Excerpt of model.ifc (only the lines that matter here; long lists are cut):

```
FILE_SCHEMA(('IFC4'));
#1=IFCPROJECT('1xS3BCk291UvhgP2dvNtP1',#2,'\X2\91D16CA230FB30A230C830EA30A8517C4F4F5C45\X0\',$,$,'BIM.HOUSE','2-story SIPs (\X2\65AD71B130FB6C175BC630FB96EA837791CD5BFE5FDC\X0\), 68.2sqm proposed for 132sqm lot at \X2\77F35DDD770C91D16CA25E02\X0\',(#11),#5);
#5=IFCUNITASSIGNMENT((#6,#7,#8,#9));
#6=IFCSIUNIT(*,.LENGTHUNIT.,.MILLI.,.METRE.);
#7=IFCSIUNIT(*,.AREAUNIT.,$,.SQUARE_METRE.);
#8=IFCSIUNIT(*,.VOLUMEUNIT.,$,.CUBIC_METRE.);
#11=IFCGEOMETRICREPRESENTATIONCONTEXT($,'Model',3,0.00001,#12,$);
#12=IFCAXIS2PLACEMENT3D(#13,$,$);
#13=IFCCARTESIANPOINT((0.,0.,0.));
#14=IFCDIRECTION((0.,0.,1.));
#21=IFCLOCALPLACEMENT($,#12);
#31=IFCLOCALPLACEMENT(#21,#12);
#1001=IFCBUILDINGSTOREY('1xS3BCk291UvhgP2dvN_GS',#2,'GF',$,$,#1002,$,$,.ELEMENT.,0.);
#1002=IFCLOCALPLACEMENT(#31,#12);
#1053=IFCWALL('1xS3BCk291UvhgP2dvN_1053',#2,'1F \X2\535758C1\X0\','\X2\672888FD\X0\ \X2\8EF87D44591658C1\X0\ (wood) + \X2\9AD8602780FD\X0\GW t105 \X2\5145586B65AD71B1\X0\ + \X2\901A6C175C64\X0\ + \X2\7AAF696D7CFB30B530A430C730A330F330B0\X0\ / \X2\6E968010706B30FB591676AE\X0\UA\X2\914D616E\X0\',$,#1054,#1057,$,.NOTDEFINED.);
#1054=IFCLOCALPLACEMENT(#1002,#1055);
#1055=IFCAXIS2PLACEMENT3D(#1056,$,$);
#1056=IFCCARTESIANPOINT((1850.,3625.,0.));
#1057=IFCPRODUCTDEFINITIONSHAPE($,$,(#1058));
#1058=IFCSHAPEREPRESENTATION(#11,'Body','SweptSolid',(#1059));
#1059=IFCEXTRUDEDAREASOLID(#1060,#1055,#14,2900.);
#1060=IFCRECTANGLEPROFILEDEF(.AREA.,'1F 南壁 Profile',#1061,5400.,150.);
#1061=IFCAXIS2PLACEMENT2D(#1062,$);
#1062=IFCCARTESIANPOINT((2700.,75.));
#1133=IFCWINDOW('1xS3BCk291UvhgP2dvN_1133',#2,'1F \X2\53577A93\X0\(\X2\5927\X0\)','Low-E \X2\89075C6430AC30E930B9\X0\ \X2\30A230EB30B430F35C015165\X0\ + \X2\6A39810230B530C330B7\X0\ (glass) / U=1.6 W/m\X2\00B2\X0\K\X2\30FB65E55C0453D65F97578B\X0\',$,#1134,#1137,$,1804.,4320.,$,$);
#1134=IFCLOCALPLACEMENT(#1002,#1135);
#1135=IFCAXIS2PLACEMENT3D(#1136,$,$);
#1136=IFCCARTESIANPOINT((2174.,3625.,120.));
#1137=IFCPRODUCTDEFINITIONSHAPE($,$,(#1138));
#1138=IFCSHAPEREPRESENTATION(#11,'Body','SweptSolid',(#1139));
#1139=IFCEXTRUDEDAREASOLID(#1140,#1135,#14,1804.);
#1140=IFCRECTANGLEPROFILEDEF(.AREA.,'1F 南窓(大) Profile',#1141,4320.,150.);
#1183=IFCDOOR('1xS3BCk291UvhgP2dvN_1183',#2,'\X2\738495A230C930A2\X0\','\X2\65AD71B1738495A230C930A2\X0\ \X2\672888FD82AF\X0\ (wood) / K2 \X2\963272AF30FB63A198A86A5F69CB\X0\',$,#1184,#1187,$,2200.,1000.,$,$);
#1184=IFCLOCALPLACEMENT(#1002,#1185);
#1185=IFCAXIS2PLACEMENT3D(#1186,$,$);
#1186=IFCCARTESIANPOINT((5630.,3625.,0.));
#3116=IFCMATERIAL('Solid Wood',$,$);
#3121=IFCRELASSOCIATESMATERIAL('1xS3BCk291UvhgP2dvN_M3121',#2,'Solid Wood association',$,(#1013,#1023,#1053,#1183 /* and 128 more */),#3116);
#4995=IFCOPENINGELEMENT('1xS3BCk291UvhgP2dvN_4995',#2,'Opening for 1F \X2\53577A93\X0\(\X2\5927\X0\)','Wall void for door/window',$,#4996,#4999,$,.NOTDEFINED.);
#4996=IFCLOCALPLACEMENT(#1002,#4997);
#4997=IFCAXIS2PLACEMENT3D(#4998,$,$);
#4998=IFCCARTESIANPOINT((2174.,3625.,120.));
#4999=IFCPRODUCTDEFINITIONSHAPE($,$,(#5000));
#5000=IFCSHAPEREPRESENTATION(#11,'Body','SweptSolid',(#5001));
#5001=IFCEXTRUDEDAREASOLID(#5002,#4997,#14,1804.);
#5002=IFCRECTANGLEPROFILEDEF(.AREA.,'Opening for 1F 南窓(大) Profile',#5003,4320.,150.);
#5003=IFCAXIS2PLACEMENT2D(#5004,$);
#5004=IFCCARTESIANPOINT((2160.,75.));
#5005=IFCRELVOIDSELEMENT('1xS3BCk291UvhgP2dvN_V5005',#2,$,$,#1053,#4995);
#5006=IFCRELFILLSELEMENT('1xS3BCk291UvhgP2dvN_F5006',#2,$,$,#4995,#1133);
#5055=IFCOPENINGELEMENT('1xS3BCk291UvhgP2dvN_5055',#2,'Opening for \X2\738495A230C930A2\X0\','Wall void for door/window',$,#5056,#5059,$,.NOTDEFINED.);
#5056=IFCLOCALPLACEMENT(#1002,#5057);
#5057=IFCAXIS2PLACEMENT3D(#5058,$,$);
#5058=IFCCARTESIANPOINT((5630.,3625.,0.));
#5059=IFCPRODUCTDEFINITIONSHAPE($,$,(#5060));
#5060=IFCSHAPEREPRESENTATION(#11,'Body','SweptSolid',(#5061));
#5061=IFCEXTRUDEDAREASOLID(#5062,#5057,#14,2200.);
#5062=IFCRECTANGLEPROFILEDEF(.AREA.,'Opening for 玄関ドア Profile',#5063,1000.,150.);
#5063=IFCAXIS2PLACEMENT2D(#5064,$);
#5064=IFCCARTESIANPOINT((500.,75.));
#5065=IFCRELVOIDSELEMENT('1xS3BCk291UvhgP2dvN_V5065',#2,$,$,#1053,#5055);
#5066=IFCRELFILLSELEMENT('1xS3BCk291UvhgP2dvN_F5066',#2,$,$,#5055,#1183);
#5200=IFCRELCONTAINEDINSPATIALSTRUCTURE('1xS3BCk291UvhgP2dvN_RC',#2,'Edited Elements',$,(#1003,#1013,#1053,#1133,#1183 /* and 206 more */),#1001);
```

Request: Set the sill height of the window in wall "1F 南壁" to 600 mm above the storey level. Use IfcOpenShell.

```python
import numpy as np
import ifcopenshell
import ifcopenshell.api.geometry
import ifcopenshell.geom
import ifcopenshell.util.element
import ifcopenshell.util.placement
import ifcopenshell.util.shape
import ifcopenshell.util.unit

model = ifcopenshell.open("model.ifc")
unit_scale = ifcopenshell.util.unit.calculate_unit_scale(model)

window = model.by_guid("1xS3BCk291UvhgP2dvN_1133")
opening = window.FillsVoids[0].RelatingOpeningElement
storey = ifcopenshell.util.element.get_container(window, ifc_class="IfcBuildingStorey")
level = ifcopenshell.util.placement.get_local_placement(storey.ObjectPlacement)[2, 3]

# The opening's origin need not be at the sill, so measure its lowest point.
shape = ifcopenshell.geom.create_shape(ifcopenshell.geom.settings(), opening)
bottom = ifcopenshell.util.shape.get_shape_bottom_elevation(shape, shape.geometry) / unit_scale
dz = level + 0.6 / unit_scale - bottom

shift = np.array([0.0, 0.0, dz])
# The window is not placed relative to its opening, so move both.
for product in (opening, window):
    matrix = ifcopenshell.util.placement.get_local_placement(product.ObjectPlacement)
    matrix[:3, 3] += shift
    ifcopenshell.api.geometry.edit_object_placement(model, product=product, matrix=matrix, is_si=False)

print(f"moved by {dz * unit_scale:+.3f} m")

model.write("model-out.ifc")
```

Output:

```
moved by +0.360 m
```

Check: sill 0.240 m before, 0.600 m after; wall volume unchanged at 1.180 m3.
